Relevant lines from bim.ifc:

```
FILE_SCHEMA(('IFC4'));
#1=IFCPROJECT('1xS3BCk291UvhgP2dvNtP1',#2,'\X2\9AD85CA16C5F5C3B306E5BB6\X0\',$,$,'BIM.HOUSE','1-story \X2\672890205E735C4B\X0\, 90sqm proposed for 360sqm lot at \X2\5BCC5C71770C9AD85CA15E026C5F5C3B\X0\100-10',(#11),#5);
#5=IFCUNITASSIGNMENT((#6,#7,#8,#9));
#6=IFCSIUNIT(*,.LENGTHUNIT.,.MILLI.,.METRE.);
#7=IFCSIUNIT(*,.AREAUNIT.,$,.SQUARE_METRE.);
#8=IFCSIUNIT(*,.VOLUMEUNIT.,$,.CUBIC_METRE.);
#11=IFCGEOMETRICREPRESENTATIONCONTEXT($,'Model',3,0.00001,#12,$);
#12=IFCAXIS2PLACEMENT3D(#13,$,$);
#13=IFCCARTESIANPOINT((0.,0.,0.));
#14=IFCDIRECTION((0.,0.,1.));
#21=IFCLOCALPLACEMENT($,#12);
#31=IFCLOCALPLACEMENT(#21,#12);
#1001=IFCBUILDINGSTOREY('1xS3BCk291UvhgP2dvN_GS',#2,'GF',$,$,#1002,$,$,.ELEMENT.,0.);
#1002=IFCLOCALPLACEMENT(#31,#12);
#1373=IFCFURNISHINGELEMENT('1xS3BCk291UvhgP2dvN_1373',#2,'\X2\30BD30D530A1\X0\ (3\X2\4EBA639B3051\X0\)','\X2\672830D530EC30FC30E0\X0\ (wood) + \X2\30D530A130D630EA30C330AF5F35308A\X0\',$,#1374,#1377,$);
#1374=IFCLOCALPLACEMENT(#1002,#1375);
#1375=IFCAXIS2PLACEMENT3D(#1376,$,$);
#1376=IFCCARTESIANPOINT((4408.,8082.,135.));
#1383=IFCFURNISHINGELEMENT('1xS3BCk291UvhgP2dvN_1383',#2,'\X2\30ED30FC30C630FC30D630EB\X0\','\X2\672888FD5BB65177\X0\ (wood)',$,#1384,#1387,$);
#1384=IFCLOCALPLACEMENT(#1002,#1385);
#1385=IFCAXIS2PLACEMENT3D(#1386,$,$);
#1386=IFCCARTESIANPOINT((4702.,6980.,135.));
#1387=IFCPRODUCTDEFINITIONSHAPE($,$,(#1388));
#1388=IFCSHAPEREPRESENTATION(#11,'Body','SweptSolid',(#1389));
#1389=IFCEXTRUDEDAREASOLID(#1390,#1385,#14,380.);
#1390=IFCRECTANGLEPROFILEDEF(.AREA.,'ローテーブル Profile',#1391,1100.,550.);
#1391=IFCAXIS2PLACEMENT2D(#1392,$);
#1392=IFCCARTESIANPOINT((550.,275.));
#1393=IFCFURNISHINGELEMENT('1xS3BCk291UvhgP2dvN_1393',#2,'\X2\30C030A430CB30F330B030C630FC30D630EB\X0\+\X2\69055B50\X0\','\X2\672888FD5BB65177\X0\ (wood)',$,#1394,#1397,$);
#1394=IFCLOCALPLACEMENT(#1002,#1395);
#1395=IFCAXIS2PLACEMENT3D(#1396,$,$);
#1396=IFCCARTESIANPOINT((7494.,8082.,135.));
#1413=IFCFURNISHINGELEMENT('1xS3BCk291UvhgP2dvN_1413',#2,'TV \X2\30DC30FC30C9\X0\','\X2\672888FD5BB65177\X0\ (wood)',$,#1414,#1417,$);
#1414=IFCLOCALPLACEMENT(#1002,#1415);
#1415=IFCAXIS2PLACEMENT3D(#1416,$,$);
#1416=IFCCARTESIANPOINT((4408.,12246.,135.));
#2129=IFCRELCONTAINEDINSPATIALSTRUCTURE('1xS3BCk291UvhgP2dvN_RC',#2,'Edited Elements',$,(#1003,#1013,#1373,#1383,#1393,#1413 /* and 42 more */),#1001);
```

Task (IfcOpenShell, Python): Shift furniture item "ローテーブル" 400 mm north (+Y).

```python
import ifcopenshell
import ifcopenshell.api.geometry
import ifcopenshell.util.placement
import ifcopenshell.util.unit

model = ifcopenshell.open("bim.ifc")
unit_scale = ifcopenshell.util.unit.calculate_unit_scale(model)

item = model.by_guid("1xS3BCk291UvhgP2dvN_1383")
matrix = ifcopenshell.util.placement.get_local_placement(item.ObjectPlacement)
matrix[1, 3] += 0.4 / unit_scale
ifcopenshell.api.geometry.edit_object_placement(model, product=item, matrix=matrix, is_si=False)

print(ifcopenshell.util.placement.get_local_placement(item.ObjectPlacement).round(3) + 0.0)

model.write("bim-out.ifc")
```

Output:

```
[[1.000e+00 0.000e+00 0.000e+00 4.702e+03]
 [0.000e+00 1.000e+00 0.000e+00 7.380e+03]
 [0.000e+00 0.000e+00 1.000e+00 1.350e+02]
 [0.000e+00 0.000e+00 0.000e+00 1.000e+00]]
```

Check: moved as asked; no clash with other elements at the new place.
